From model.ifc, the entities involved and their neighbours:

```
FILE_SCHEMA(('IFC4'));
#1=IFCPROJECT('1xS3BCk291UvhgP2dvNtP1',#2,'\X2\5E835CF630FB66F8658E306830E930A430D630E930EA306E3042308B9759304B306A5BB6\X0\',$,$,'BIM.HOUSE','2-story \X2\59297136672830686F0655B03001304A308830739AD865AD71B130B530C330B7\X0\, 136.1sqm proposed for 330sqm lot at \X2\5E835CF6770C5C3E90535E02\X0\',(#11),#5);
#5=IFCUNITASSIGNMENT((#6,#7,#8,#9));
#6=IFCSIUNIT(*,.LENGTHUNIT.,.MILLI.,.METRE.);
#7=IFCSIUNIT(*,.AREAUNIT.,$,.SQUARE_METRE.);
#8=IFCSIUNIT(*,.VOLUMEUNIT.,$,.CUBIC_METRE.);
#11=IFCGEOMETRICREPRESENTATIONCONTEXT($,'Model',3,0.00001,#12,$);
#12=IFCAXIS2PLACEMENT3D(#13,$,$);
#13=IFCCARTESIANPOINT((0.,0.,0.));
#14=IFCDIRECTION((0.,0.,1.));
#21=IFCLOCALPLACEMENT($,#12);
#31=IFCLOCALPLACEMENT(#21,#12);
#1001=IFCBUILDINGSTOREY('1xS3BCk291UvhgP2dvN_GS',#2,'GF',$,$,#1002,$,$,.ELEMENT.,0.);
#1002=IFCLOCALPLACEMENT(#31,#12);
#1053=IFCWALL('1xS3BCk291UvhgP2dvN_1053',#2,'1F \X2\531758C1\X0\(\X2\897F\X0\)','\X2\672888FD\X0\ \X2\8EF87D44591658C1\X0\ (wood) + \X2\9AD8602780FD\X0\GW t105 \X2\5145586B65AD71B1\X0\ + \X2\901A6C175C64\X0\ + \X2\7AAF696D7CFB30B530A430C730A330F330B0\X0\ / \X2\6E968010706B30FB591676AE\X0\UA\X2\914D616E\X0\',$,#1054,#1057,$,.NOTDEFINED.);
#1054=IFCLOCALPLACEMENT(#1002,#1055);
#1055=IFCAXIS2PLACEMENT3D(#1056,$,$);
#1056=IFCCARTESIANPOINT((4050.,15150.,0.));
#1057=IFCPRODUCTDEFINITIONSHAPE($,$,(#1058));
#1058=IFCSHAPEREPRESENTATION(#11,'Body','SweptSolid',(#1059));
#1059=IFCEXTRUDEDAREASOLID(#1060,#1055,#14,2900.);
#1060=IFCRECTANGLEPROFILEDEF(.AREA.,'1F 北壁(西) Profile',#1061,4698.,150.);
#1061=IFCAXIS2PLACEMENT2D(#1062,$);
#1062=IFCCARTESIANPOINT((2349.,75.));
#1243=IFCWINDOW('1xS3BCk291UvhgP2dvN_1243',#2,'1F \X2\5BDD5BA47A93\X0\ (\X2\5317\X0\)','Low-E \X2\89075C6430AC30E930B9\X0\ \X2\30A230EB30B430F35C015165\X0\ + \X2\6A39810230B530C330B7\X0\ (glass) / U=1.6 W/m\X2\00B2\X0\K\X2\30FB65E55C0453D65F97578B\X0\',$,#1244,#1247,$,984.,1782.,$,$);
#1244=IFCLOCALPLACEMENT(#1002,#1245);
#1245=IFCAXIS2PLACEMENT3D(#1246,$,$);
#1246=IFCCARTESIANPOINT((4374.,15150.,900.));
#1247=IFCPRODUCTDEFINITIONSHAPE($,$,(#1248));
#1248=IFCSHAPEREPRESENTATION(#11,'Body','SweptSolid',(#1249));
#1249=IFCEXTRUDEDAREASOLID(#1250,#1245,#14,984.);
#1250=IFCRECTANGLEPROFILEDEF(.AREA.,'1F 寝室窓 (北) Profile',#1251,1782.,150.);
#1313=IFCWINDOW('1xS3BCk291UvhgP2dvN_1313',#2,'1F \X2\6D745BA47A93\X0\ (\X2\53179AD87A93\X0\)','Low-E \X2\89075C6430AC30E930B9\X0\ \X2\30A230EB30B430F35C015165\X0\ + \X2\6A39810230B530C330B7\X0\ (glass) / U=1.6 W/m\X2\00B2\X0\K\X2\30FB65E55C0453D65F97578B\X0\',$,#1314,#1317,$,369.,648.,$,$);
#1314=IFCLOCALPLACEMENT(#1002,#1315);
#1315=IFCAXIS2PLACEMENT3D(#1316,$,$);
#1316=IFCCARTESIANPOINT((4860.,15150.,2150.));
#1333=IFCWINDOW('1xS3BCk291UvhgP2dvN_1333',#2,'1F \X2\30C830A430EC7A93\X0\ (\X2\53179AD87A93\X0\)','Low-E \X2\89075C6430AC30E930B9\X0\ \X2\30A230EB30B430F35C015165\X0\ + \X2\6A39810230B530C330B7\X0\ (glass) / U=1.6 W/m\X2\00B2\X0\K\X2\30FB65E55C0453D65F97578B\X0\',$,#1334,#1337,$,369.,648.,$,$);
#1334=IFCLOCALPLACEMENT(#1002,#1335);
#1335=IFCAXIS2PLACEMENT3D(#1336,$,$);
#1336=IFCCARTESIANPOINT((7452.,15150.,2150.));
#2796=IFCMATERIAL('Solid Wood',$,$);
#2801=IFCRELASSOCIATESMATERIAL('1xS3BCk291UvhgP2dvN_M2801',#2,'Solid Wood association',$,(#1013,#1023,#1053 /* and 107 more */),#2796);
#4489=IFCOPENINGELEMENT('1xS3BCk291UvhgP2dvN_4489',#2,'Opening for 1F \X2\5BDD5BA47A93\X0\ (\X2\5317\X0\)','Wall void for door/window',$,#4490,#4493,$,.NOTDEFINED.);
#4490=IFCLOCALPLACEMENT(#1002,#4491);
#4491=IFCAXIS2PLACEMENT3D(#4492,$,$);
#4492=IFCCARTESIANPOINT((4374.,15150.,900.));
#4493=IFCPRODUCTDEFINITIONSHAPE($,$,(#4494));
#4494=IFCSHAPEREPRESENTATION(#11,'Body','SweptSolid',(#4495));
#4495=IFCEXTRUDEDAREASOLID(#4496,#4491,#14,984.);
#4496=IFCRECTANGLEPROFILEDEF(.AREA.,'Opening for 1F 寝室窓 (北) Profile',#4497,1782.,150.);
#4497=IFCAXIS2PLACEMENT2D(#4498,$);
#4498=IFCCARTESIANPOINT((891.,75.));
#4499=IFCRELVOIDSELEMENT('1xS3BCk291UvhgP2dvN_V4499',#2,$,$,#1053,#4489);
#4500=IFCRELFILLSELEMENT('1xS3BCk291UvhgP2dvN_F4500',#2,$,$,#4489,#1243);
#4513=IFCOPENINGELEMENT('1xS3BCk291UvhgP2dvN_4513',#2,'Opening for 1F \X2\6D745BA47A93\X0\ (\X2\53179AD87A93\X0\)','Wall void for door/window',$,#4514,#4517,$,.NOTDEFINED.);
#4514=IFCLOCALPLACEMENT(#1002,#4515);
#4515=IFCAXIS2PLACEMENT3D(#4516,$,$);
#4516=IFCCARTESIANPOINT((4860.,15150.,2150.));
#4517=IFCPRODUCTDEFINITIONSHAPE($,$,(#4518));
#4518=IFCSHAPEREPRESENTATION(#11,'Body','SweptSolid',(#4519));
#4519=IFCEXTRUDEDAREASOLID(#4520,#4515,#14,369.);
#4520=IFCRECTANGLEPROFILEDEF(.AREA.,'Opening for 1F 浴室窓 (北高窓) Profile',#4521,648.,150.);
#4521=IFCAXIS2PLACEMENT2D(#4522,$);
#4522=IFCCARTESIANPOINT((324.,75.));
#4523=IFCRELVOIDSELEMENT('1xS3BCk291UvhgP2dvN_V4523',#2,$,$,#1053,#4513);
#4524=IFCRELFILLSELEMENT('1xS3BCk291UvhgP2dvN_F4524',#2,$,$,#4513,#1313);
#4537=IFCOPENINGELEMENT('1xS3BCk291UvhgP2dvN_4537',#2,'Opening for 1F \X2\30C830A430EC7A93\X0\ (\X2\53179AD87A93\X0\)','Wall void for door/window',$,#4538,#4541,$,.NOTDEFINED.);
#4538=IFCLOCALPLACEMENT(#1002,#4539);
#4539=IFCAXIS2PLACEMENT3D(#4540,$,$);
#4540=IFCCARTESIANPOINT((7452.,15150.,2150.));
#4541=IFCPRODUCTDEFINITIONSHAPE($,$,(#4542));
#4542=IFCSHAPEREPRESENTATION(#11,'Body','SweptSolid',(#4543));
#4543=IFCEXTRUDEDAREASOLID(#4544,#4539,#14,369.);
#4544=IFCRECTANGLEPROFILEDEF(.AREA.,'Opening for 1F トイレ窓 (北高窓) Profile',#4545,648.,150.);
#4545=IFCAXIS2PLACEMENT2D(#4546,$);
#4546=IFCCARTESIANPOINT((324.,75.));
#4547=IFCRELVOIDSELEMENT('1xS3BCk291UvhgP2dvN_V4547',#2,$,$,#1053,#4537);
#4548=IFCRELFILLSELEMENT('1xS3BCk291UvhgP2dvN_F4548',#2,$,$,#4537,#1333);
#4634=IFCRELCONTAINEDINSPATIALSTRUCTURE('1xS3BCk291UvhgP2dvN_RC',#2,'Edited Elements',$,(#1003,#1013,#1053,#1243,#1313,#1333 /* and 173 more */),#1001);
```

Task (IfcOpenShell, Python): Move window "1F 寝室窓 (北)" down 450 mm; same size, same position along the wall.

```python
import numpy as np
import ifcopenshell
import ifcopenshell.api.geometry
import ifcopenshell.util.placement
import ifcopenshell.util.unit

model = ifcopenshell.open("model.ifc")
unit_scale = ifcopenshell.util.unit.calculate_unit_scale(model)

window = model.by_id(1243)
opening = window.FillsVoids[0].RelatingOpeningElement
dz = -0.45 / unit_scale

shift = np.array([0.0, 0.0, dz])
# The window is not placed relative to its opening, so move both.
for product in (opening, window):
    matrix = ifcopenshell.util.placement.get_local_placement(product.ObjectPlacement)
    matrix[:3, 3] += shift
    ifcopenshell.api.geometry.edit_object_placement(model, product=product, matrix=matrix, is_si=False)

print(f"moved by {dz * unit_scale:+.3f} m")

model.write("model_v2.ifc")
```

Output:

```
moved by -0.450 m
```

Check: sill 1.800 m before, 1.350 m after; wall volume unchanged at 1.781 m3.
